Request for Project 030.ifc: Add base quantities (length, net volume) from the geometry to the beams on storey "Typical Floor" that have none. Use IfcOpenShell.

First a look at what the model holds.

```python
import ifcopenshell
import ifcopenshell.util.element
import ifcopenshell.util.unit

model = ifcopenshell.open("Project 030.ifc")
print(model.schema)
for unit_type in ("LENGTHUNIT", "AREAUNIT", "VOLUMEUNIT"):
    print(unit_type, ifcopenshell.util.unit.calculate_unit_scale(model, unit_type))
storey = next(s for s in model.by_type("IfcBuildingStorey") if s.Name == "Typical Floor")
beams = [e for e in ifcopenshell.util.element.get_decomposition(storey) if e.is_a("IfcBeam")]
for e in sorted(beams, key=lambda e: e.id()):
    print(e.id(), e.is_a(), e.Name, list(ifcopenshell.util.element.get_psets(e, qtos_only=True)), sep=" | ")
```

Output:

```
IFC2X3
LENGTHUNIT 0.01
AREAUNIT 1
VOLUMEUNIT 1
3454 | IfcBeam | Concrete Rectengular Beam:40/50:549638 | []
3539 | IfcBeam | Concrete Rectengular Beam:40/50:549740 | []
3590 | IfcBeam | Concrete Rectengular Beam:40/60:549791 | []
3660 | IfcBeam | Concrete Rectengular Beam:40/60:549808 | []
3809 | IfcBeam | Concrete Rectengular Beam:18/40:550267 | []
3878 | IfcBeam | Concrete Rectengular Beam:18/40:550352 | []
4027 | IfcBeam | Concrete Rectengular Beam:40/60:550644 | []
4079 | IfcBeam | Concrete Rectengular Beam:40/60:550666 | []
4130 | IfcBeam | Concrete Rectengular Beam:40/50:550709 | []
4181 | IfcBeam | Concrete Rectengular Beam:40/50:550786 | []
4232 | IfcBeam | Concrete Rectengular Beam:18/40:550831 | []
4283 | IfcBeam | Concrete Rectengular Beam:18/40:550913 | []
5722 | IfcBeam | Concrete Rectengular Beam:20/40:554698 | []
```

```python
import ifcopenshell
import ifcopenshell.api.pset
import ifcopenshell.geom
import ifcopenshell.util.element
import ifcopenshell.util.shape
import ifcopenshell.util.unit

model = ifcopenshell.open("Project 030.ifc")
unit_scale = ifcopenshell.util.unit.calculate_unit_scale(model)
volume_scale = ifcopenshell.util.unit.calculate_unit_scale(model, "VOLUMEUNIT")
settings = ifcopenshell.geom.settings()

storey = next(s for s in model.by_type("IfcBuildingStorey") if s.Name == "Typical Floor")
beams = [e for e in ifcopenshell.util.element.get_decomposition(storey) if e.is_a("IfcBeam")]

for e in sorted(beams, key=lambda e: e.id()):
    if ifcopenshell.util.element.get_psets(e, qtos_only=True, should_inherit=False):
        continue
    # Geometry comes back in metres, in the element's own axes.
    shape = ifcopenshell.geom.create_shape(settings, e)
    values = {
        "Length": ifcopenshell.util.shape.get_max_xyz(shape.geometry) / unit_scale,
        "NetVolume": ifcopenshell.util.shape.get_volume(shape.geometry) / volume_scale,
    }
    qto = ifcopenshell.api.pset.add_qto(model, product=e, name="BaseQuantities")
    ifcopenshell.api.pset.edit_qto(model, qto=qto, properties=values)
    print(e.id(), {k: round(v, 3) for k, v in values.items()})

model.write("Project 030_updated.ifc")
```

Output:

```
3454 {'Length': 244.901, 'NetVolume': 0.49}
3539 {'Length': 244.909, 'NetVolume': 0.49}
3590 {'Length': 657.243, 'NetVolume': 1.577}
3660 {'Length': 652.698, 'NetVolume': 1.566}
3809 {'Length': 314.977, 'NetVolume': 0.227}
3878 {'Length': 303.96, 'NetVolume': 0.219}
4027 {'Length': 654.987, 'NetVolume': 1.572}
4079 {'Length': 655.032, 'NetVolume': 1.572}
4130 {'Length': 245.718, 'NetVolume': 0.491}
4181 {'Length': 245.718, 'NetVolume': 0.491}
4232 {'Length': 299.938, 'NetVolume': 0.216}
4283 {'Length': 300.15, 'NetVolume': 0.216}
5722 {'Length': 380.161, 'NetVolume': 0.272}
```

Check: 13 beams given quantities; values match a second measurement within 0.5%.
